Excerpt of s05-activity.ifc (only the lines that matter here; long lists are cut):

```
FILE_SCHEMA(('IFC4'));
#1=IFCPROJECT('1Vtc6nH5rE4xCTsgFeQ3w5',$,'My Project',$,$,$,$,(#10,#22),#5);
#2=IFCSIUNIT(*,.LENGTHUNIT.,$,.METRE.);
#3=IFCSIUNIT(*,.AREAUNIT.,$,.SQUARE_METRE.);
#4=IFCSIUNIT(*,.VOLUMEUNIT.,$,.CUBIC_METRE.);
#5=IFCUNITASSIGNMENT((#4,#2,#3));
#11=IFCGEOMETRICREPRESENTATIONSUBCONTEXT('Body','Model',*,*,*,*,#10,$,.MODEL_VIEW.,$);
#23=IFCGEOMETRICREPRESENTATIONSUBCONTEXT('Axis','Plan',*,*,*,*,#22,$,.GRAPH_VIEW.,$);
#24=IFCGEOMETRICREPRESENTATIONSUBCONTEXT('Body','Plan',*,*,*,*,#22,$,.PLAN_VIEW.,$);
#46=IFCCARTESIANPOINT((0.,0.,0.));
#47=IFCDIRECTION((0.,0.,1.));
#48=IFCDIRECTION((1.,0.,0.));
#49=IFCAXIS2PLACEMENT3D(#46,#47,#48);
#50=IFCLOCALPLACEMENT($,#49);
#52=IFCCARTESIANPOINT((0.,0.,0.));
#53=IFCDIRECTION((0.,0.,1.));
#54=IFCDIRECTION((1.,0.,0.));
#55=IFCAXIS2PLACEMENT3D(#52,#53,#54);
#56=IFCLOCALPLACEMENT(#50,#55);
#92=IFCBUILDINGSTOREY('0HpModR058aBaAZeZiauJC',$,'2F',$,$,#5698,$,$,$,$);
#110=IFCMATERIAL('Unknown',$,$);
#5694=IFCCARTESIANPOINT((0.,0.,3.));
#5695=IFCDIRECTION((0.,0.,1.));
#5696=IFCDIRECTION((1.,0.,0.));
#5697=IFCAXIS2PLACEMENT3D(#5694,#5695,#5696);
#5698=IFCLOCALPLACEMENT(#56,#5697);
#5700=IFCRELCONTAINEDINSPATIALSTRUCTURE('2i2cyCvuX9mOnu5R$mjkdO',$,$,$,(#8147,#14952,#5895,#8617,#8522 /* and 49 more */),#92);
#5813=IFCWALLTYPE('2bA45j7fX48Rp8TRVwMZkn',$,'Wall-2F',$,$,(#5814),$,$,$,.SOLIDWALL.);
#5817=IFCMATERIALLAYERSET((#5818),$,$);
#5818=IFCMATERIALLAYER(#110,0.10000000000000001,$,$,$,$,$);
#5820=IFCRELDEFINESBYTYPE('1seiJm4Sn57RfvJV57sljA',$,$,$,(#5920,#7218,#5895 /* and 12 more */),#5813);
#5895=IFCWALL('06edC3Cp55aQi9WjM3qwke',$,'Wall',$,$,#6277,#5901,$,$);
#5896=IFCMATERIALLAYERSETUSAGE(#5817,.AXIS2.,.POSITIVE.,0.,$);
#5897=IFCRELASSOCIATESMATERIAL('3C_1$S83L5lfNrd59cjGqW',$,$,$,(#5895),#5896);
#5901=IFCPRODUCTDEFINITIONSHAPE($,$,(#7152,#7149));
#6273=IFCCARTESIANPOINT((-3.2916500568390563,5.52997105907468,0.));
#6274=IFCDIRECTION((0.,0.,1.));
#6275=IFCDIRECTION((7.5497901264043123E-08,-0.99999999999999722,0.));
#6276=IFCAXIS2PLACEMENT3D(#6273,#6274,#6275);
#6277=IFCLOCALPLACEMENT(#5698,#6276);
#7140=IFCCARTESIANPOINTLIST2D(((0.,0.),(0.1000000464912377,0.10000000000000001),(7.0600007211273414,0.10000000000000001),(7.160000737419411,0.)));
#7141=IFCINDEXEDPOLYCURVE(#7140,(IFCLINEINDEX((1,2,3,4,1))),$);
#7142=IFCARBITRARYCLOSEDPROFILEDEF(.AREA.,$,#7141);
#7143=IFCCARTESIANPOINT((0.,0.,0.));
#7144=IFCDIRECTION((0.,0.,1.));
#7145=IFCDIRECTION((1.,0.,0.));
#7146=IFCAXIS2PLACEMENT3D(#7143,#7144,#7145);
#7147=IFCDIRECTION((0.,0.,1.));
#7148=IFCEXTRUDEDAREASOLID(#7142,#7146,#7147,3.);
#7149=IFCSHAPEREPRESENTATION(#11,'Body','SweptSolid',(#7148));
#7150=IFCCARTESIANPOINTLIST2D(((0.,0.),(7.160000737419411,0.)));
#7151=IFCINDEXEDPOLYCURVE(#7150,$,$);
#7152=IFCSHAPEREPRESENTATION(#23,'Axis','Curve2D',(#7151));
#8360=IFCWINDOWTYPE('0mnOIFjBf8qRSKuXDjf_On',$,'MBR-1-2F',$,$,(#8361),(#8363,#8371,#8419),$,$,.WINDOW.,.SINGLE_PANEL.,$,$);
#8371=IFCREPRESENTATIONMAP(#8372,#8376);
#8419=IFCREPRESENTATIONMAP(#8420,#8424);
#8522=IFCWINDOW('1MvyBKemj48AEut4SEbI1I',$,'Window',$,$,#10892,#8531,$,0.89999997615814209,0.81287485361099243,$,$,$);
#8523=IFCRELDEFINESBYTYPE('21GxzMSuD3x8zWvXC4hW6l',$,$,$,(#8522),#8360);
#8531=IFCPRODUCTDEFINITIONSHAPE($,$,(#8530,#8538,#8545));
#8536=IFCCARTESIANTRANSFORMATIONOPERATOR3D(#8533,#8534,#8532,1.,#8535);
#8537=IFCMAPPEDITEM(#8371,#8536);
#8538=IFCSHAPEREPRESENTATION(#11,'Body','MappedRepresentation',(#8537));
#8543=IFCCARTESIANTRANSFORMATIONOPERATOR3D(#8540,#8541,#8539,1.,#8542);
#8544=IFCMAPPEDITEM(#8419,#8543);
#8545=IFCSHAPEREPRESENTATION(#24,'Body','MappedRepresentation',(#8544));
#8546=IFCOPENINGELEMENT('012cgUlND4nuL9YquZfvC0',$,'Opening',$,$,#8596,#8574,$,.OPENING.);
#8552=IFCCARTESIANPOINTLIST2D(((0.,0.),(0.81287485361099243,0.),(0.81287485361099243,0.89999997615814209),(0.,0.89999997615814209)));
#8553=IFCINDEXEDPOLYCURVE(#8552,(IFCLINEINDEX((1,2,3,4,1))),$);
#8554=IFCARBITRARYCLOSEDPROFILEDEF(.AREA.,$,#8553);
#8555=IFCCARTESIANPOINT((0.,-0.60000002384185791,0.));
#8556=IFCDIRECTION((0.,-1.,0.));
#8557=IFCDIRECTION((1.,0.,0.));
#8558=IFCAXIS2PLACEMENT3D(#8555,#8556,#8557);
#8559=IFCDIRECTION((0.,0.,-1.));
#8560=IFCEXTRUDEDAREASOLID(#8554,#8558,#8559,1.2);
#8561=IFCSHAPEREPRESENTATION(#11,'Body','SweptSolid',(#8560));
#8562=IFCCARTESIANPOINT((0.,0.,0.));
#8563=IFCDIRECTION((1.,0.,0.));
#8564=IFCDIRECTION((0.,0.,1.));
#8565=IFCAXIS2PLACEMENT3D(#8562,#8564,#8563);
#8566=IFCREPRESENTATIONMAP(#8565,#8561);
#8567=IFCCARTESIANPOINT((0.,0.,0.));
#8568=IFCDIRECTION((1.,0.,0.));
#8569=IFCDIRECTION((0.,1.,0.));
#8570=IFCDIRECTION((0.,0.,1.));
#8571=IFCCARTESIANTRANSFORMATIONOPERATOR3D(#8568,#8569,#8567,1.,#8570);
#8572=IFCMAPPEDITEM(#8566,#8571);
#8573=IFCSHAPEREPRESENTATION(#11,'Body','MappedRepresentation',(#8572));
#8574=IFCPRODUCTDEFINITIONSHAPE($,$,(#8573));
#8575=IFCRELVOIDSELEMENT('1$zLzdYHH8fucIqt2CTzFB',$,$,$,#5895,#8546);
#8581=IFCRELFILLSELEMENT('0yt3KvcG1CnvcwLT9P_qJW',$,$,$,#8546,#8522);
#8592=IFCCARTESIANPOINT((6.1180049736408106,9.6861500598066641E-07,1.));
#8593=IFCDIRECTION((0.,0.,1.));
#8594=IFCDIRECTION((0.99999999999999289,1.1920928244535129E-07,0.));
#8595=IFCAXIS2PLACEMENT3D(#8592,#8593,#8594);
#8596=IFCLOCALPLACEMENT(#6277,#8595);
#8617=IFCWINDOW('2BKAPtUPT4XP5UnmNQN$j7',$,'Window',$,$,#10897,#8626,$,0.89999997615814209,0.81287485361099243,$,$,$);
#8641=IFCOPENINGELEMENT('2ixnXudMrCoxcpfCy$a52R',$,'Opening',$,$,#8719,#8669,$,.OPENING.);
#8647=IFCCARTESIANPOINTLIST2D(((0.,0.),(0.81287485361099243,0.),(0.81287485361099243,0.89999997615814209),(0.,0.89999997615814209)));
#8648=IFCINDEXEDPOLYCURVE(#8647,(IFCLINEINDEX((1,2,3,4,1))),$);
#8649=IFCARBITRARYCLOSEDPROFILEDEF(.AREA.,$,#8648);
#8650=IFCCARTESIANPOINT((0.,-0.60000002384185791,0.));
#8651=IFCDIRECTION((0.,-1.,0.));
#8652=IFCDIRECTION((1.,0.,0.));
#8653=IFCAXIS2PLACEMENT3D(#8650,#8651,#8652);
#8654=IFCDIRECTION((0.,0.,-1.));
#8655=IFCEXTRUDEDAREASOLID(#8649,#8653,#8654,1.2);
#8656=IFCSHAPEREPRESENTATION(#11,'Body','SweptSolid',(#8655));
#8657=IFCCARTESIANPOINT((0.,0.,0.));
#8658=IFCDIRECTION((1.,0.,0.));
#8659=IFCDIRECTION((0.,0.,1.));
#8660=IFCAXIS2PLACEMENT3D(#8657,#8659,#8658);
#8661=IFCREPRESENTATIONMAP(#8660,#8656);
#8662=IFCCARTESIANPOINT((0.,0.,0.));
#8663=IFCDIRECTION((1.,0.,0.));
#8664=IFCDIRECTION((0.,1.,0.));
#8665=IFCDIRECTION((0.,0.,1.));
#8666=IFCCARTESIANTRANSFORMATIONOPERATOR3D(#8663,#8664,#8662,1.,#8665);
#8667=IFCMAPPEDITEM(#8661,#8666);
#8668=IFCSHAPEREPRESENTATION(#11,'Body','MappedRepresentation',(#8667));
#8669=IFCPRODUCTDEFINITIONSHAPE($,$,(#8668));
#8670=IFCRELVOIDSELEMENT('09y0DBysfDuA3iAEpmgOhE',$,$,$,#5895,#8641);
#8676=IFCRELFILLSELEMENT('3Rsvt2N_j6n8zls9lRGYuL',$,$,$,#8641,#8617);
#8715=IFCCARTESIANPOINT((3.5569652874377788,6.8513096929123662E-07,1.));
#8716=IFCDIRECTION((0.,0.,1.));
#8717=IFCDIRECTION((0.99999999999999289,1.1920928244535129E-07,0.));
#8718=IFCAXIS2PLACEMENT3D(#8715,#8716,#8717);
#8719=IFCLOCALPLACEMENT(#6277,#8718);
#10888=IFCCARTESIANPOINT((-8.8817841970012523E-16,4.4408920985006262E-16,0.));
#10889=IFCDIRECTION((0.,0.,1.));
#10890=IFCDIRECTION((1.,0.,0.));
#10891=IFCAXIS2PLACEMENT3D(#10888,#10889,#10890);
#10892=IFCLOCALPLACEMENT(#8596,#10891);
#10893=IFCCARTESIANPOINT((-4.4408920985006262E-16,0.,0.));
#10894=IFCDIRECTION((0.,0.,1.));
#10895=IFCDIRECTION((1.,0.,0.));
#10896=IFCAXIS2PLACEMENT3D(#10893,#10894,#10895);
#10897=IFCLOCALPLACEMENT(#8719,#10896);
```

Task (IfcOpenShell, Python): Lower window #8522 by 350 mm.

```python
import numpy as np
import ifcopenshell
import ifcopenshell.api.geometry
import ifcopenshell.util.placement
import ifcopenshell.util.unit

model = ifcopenshell.open("s05-activity.ifc")
unit_scale = ifcopenshell.util.unit.calculate_unit_scale(model)

window = model.by_guid("1MvyBKemj48AEut4SEbI1I")
opening = window.FillsVoids[0].RelatingOpeningElement
dz = -0.35 / unit_scale

shift = np.array([0.0, 0.0, dz])
# The window is placed relative to its opening, so it follows when the opening moves.
matrix = ifcopenshell.util.placement.get_local_placement(opening.ObjectPlacement)
matrix[:3, 3] += shift
ifcopenshell.api.geometry.edit_object_placement(
    model, product=opening, matrix=matrix, is_si=False, should_transform_children=True
)

print(f"moved by {dz * unit_scale:+.3f} m")

model.write("s05-activity-out.ifc")
```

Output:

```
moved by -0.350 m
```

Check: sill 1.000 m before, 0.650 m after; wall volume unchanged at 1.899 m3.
